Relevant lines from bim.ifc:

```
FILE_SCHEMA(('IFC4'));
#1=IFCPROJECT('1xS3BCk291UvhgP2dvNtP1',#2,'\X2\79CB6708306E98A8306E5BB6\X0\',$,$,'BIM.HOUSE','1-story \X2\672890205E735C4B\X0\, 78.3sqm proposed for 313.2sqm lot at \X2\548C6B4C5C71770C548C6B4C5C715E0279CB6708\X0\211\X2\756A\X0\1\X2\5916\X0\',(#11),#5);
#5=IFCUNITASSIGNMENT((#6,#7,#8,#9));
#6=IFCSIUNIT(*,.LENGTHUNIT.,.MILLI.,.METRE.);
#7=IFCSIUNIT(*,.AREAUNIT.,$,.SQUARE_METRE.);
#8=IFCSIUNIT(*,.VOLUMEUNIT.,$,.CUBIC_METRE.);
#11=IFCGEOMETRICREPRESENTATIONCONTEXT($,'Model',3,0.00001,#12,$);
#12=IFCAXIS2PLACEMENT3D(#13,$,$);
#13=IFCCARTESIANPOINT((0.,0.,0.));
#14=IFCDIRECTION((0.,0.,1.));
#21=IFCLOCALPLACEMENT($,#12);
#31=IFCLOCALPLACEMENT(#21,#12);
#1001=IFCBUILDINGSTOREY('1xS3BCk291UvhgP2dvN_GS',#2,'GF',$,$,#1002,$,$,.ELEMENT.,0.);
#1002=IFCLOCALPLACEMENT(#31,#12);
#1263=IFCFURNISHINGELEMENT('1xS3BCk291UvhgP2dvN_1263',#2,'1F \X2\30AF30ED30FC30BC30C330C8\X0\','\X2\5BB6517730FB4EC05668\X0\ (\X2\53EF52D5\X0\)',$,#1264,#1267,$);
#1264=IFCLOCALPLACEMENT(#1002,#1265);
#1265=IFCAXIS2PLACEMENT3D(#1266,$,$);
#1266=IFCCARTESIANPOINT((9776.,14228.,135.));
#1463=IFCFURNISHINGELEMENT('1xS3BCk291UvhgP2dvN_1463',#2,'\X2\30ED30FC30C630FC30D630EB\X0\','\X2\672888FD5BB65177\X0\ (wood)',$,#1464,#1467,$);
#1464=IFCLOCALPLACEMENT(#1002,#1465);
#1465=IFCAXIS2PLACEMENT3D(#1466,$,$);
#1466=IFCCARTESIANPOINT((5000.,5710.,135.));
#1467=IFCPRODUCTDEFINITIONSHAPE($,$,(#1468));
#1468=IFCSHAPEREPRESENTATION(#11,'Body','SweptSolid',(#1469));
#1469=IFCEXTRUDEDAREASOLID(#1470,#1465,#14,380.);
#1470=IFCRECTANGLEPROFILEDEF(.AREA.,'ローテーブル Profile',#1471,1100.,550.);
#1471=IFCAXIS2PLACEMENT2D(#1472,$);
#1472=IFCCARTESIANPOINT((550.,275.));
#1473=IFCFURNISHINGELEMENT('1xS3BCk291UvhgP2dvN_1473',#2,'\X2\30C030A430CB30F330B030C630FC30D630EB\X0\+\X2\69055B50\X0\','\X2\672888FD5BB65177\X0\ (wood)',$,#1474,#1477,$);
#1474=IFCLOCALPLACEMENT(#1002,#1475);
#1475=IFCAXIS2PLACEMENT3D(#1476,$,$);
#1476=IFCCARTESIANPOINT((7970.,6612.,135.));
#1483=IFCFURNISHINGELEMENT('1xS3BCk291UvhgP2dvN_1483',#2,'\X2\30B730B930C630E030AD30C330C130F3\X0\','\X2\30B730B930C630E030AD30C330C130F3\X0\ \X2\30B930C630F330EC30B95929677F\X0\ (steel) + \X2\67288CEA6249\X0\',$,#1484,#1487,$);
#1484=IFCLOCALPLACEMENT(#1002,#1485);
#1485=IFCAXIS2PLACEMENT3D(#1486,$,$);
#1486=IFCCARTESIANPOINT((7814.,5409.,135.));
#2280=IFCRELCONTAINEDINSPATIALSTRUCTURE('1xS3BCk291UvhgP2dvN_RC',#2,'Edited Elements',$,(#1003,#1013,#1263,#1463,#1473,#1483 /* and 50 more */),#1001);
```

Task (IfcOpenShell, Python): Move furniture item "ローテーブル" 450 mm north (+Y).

```python
import ifcopenshell
import ifcopenshell.api.geometry
import ifcopenshell.util.placement
import ifcopenshell.util.unit

model = ifcopenshell.open("bim.ifc")
unit_scale = ifcopenshell.util.unit.calculate_unit_scale(model)

item = model.by_guid("1xS3BCk291UvhgP2dvN_1463")
matrix = ifcopenshell.util.placement.get_local_placement(item.ObjectPlacement)
matrix[1, 3] += 0.45 / unit_scale
ifcopenshell.api.geometry.edit_object_placement(model, product=item, matrix=matrix, is_si=False)

print(ifcopenshell.util.placement.get_local_placement(item.ObjectPlacement).round(3) + 0.0)

model.write("bim_updated.ifc")
```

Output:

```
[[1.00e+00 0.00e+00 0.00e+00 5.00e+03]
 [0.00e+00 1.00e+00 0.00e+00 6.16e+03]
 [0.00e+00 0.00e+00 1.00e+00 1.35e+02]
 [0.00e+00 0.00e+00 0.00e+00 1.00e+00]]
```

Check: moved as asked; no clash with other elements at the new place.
